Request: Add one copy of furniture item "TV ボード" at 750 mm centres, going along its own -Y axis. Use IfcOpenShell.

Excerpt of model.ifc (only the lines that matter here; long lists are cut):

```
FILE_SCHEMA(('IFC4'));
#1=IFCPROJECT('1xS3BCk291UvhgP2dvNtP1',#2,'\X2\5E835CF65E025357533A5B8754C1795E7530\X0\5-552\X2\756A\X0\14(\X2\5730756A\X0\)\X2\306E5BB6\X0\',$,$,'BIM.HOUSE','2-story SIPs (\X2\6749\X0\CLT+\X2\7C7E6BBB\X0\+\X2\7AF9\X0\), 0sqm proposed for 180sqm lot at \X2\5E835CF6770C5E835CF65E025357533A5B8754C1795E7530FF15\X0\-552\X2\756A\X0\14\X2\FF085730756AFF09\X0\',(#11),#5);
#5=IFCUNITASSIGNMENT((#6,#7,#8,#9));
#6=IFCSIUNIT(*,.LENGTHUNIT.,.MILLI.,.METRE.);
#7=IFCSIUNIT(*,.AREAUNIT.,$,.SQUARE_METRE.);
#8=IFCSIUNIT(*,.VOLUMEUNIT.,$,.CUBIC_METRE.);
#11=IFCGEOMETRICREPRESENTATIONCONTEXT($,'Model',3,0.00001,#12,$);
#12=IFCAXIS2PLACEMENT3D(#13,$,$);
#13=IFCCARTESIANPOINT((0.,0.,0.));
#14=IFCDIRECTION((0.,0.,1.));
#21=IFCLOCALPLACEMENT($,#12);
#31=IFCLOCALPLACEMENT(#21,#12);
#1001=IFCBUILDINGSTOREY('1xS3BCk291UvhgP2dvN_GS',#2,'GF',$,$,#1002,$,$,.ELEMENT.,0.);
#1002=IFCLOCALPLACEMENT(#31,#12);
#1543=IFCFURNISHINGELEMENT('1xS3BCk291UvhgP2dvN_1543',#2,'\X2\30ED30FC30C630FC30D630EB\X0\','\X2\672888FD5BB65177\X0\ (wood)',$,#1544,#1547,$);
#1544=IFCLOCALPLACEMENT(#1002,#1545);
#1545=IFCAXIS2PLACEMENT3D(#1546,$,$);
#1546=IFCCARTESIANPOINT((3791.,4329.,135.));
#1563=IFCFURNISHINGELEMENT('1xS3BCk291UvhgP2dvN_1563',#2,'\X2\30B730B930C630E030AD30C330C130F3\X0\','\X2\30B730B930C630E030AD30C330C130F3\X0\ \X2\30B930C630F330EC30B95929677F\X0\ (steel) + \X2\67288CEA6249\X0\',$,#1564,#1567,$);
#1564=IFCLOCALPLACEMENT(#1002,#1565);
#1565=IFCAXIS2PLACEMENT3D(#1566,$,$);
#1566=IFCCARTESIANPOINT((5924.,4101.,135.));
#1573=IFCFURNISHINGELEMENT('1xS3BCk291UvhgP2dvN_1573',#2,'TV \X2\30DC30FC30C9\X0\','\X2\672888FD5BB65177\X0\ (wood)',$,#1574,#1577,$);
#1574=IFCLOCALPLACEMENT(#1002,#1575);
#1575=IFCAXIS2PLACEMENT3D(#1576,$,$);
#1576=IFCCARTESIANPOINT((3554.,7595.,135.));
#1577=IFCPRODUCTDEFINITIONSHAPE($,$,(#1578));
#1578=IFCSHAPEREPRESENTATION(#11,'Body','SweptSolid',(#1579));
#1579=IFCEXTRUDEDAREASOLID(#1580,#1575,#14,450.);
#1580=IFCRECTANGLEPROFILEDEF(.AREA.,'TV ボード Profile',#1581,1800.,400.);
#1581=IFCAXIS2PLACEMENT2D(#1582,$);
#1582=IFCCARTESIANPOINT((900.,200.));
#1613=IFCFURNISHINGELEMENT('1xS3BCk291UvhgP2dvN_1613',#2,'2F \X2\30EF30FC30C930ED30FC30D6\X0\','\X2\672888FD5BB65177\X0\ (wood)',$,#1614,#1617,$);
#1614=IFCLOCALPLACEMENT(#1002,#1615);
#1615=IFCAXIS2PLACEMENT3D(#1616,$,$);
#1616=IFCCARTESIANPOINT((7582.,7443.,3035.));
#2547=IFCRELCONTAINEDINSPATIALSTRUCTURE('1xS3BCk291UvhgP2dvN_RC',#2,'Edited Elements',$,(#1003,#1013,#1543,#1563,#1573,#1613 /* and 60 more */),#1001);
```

```python
import ifcopenshell
import ifcopenshell.api.geometry
import ifcopenshell.api.root
import ifcopenshell.util.element
import ifcopenshell.util.placement
import ifcopenshell.util.unit

model = ifcopenshell.open("model.ifc")
unit_scale = ifcopenshell.util.unit.calculate_unit_scale(model)


def reuse_history(source, copy):
    """copy_class also copies each property set's owner history, people and application; keep the originals."""
    for rel in copy.IsDefinedBy:
        if rel.is_a("IfcRelDefinesByProperties") and (history := rel.RelatingPropertyDefinition.OwnerHistory):
            rel.RelatingPropertyDefinition.OwnerHistory = source.OwnerHistory
            ifcopenshell.util.element.remove_deep2(model, history)


source = model.by_guid("1xS3BCk291UvhgP2dvN_1573")
base = ifcopenshell.util.placement.get_local_placement(source.ObjectPlacement)
step = -base[:3, 1] * 0.75 / unit_scale

for i in range(1, 2):
    copy = ifcopenshell.api.root.copy_class(model, product=source)
    copy.Representation = ifcopenshell.util.element.copy_deep(
        model, source.Representation, exclude=["IfcGeometricRepresentationContext", "IfcRepresentationMap"]
    )
    reuse_history(source, copy)
    matrix = base.copy()
    matrix[:3, 3] += i * step
    print("added at", matrix[:3, 3].round(3) + 0.0)
    ifcopenshell.api.geometry.edit_object_placement(model, product=copy, matrix=matrix, is_si=False)

model.write("model_updated.ifc")
```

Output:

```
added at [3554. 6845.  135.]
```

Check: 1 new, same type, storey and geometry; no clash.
